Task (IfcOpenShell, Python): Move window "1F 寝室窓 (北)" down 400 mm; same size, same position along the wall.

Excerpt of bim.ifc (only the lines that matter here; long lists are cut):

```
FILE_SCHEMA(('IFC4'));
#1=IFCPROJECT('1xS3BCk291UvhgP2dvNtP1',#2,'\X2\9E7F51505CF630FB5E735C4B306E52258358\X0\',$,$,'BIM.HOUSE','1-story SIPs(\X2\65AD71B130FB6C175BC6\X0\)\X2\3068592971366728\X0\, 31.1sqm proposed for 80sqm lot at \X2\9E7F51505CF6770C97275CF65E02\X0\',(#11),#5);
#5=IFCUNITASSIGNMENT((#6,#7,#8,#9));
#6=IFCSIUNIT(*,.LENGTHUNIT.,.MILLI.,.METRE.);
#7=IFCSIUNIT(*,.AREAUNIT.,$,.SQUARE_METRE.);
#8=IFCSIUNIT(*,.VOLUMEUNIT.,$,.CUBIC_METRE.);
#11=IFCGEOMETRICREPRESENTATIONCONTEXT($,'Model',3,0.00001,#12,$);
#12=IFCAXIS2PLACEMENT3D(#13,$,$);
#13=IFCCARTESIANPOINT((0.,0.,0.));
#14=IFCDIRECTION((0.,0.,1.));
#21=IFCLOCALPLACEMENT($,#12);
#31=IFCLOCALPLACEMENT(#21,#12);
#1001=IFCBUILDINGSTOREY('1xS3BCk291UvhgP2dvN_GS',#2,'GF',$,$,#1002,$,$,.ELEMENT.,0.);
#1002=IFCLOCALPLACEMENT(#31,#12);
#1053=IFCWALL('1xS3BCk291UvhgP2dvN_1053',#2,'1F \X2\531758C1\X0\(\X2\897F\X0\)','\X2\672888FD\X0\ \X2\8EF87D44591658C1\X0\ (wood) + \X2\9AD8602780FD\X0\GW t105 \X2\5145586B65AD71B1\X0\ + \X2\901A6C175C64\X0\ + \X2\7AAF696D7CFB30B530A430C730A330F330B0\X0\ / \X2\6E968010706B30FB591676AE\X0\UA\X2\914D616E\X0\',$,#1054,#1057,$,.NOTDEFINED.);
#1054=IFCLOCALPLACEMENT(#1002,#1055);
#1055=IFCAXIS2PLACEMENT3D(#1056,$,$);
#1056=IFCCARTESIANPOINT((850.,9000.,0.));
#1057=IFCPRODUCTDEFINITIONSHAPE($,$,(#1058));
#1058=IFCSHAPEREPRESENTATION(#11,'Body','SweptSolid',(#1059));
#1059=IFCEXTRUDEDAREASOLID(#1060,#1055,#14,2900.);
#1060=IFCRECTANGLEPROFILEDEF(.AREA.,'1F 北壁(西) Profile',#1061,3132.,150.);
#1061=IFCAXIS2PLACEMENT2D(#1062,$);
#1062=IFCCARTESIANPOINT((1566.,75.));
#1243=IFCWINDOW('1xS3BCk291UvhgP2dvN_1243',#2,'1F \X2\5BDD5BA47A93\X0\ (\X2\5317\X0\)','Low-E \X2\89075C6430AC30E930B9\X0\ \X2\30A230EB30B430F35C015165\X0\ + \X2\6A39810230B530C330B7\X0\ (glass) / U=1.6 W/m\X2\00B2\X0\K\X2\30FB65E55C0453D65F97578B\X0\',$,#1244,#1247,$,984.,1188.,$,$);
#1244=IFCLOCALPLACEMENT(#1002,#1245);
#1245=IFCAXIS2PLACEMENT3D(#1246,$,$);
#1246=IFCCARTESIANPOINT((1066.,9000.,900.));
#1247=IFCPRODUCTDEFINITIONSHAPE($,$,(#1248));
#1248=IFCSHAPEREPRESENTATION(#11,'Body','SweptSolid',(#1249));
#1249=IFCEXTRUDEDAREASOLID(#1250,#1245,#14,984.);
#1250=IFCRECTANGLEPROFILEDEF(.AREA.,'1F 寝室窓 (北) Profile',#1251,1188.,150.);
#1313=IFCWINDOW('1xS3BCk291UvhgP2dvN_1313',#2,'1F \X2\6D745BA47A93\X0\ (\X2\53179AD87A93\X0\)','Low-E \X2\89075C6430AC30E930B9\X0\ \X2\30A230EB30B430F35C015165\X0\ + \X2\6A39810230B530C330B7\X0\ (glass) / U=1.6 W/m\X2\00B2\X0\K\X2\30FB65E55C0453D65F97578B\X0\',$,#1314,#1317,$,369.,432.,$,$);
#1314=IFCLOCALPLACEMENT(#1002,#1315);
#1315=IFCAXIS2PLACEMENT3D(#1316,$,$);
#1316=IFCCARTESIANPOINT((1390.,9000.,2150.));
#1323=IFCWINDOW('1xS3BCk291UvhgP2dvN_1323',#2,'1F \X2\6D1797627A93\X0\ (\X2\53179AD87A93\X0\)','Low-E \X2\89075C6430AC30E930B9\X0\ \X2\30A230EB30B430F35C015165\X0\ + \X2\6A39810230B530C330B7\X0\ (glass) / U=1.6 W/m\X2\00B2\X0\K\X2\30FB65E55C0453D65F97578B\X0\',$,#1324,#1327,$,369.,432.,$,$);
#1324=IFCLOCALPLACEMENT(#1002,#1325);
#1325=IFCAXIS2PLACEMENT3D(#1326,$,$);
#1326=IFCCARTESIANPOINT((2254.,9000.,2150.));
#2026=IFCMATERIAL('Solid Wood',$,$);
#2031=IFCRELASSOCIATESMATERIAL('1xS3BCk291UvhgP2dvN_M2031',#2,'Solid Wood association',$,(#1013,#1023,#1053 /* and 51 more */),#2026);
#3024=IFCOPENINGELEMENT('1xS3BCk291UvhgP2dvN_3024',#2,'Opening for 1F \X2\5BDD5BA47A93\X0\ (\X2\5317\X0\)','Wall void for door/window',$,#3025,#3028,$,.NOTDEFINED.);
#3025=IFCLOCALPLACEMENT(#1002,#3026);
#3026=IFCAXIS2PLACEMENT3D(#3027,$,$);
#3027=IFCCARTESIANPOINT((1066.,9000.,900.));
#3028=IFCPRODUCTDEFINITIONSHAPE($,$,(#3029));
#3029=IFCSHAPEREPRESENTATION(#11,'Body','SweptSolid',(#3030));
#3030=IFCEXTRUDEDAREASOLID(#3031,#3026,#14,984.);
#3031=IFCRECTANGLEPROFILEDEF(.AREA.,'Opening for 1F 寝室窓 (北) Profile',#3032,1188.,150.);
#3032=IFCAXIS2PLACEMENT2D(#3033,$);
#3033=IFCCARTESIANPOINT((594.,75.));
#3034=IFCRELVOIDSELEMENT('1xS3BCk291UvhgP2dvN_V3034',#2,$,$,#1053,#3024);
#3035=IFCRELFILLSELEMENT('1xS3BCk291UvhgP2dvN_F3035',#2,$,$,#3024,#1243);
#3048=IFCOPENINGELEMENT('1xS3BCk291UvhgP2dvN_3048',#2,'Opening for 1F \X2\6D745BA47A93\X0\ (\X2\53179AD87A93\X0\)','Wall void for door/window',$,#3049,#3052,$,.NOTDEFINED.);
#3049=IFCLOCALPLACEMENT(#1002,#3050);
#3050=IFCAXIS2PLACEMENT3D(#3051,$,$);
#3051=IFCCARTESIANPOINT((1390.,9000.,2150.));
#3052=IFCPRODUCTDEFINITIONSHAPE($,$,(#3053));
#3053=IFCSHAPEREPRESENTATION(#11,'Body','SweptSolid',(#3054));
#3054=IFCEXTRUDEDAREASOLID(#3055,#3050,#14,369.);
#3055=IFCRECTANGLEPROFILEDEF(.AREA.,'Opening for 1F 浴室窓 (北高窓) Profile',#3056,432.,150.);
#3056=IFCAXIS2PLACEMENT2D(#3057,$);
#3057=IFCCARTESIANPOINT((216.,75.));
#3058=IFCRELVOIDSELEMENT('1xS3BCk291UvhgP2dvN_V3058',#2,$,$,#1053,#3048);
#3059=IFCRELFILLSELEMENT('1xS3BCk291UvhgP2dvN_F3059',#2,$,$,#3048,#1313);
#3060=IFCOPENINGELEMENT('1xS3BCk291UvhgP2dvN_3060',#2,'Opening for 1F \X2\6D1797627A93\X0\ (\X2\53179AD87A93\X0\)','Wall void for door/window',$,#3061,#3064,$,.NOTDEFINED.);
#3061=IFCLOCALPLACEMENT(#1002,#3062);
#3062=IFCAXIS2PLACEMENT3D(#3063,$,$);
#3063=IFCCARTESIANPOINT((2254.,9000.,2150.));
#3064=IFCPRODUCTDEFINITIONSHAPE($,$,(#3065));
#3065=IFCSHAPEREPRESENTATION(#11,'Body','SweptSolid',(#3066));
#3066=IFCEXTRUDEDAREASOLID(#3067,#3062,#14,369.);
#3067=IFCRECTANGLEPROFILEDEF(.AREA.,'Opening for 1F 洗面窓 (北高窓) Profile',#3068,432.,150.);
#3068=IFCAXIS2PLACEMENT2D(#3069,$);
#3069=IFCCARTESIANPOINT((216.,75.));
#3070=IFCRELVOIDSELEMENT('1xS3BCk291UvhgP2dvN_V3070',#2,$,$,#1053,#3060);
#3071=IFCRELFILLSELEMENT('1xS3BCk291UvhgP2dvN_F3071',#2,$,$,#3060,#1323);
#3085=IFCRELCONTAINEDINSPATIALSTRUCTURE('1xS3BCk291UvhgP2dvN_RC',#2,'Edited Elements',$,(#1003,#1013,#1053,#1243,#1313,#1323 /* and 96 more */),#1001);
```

```python
import numpy as np
import ifcopenshell
import ifcopenshell.api.geometry
import ifcopenshell.util.placement
import ifcopenshell.util.unit

model = ifcopenshell.open("bim.ifc")
unit_scale = ifcopenshell.util.unit.calculate_unit_scale(model)

window = model.by_guid("1xS3BCk291UvhgP2dvN_1243")
opening = window.FillsVoids[0].RelatingOpeningElement
dz = -0.4 / unit_scale

shift = np.array([0.0, 0.0, dz])
# The window is not placed relative to its opening, so move both.
for product in (opening, window):
    matrix = ifcopenshell.util.placement.get_local_placement(product.ObjectPlacement)
    matrix[:3, 3] += shift
    ifcopenshell.api.geometry.edit_object_placement(model, product=product, matrix=matrix, is_si=False)

print(f"moved by {dz * unit_scale:+.3f} m")

model.write("bim-out.ifc")
```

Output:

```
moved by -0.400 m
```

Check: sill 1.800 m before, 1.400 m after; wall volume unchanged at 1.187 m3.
